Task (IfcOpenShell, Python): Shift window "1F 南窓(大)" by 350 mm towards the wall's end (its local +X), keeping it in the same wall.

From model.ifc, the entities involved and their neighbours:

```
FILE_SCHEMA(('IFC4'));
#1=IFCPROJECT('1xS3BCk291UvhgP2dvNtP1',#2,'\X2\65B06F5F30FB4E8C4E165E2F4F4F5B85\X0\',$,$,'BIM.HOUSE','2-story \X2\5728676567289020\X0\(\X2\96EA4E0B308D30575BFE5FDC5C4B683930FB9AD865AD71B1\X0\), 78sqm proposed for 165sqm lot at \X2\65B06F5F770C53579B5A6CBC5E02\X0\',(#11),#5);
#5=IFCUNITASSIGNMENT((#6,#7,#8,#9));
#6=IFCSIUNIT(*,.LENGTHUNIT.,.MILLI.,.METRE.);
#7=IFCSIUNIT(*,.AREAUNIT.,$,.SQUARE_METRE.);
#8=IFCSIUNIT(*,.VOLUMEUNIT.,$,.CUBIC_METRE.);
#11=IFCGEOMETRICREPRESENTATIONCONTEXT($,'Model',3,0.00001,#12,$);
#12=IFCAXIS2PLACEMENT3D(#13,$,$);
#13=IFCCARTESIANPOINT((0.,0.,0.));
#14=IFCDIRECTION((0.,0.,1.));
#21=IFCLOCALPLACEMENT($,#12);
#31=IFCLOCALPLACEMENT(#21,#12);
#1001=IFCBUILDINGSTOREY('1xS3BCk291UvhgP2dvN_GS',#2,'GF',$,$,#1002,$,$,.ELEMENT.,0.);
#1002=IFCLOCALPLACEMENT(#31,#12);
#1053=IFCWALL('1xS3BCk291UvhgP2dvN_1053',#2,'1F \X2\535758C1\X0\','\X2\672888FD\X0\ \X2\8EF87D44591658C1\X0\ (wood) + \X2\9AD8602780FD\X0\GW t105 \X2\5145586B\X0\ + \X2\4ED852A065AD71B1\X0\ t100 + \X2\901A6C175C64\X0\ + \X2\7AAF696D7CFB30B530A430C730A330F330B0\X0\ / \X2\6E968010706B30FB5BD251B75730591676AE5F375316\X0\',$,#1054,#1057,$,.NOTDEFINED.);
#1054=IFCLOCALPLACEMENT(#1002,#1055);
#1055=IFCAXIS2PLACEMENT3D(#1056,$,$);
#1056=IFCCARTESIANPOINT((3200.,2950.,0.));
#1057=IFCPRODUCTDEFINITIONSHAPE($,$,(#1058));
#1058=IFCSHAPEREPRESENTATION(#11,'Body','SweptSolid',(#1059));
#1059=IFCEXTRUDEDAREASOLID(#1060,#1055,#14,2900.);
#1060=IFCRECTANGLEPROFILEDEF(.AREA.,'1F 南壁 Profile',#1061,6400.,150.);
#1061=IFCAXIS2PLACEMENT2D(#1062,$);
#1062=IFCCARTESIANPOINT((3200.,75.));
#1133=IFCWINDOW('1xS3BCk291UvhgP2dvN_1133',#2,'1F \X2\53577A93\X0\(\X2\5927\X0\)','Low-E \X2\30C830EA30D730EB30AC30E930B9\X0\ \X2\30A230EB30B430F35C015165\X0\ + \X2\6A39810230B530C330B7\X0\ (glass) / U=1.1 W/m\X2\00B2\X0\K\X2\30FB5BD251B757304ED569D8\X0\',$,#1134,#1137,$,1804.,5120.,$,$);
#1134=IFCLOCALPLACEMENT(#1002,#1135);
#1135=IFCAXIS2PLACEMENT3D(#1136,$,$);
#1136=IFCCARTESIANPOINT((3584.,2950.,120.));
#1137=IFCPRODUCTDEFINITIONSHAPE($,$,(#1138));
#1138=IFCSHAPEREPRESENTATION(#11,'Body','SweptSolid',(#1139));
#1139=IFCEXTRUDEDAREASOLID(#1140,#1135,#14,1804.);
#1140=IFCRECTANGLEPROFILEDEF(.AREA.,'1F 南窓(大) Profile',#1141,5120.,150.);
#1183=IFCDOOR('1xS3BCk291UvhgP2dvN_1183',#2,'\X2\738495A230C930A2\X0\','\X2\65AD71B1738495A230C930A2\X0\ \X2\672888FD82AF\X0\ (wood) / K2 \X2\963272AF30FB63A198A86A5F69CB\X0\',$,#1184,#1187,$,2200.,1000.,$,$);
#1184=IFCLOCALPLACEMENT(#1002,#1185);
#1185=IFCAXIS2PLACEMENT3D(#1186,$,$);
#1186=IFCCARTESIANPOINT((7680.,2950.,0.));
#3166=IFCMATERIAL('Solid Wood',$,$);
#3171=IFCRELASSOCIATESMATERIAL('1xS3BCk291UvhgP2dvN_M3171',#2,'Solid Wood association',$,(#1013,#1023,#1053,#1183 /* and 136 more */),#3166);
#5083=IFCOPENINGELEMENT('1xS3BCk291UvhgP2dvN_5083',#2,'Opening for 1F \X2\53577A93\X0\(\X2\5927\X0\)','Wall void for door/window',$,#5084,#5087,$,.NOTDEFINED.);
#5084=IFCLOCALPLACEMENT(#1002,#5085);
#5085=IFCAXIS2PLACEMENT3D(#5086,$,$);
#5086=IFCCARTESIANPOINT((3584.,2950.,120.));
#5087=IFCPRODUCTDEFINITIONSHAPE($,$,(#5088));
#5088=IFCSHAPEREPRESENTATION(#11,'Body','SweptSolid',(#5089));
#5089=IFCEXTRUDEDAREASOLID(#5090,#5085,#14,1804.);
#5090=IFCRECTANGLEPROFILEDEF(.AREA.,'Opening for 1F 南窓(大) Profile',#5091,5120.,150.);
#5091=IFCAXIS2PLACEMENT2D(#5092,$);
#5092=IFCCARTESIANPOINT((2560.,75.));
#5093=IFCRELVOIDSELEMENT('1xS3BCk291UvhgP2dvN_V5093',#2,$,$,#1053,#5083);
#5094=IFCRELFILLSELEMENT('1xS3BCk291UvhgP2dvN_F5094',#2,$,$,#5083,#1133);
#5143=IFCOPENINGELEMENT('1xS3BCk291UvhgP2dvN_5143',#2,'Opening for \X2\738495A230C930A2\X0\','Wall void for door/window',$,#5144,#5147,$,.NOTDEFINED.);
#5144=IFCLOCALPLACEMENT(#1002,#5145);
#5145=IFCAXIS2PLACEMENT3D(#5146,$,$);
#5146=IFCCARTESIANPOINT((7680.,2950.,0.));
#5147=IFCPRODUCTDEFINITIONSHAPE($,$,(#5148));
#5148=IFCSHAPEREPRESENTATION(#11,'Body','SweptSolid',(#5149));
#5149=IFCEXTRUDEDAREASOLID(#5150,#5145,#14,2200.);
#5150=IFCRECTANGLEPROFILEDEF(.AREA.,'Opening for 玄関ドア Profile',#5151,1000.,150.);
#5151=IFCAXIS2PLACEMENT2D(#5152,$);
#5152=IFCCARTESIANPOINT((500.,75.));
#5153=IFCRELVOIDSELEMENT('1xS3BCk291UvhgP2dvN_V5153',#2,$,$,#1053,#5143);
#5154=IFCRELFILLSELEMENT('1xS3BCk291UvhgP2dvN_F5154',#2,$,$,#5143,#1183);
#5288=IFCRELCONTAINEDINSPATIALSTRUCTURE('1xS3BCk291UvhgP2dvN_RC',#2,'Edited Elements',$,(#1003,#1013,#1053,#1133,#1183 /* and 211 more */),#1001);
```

```python
import ifcopenshell
import ifcopenshell.api.geometry
import ifcopenshell.util.placement

model = ifcopenshell.open("model.ifc")

window = model.by_id(1133)
opening = window.FillsVoids[0].RelatingOpeningElement
wall = opening.VoidsElements[0].RelatingBuildingElement

wall_matrix = ifcopenshell.util.placement.get_local_placement(wall.ObjectPlacement)
shift = wall_matrix[:3, 0] * 350.0
before = ifcopenshell.util.placement.get_local_placement(window.ObjectPlacement)[:3, 3].copy()

# The window is not placed relative to its opening, so move both.
for product in (opening, window):
    matrix = ifcopenshell.util.placement.get_local_placement(product.ObjectPlacement)
    matrix[:3, 3] += shift
    ifcopenshell.api.geometry.edit_object_placement(model, product=product, matrix=matrix, is_si=False)

after = ifcopenshell.util.placement.get_local_placement(window.ObjectPlacement)[:3, 3]
print("window moved by", (after - before).round(3) + 0.0)

model.write("model_edited.ifc")
```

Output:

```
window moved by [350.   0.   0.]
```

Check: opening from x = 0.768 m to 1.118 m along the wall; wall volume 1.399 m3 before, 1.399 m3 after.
